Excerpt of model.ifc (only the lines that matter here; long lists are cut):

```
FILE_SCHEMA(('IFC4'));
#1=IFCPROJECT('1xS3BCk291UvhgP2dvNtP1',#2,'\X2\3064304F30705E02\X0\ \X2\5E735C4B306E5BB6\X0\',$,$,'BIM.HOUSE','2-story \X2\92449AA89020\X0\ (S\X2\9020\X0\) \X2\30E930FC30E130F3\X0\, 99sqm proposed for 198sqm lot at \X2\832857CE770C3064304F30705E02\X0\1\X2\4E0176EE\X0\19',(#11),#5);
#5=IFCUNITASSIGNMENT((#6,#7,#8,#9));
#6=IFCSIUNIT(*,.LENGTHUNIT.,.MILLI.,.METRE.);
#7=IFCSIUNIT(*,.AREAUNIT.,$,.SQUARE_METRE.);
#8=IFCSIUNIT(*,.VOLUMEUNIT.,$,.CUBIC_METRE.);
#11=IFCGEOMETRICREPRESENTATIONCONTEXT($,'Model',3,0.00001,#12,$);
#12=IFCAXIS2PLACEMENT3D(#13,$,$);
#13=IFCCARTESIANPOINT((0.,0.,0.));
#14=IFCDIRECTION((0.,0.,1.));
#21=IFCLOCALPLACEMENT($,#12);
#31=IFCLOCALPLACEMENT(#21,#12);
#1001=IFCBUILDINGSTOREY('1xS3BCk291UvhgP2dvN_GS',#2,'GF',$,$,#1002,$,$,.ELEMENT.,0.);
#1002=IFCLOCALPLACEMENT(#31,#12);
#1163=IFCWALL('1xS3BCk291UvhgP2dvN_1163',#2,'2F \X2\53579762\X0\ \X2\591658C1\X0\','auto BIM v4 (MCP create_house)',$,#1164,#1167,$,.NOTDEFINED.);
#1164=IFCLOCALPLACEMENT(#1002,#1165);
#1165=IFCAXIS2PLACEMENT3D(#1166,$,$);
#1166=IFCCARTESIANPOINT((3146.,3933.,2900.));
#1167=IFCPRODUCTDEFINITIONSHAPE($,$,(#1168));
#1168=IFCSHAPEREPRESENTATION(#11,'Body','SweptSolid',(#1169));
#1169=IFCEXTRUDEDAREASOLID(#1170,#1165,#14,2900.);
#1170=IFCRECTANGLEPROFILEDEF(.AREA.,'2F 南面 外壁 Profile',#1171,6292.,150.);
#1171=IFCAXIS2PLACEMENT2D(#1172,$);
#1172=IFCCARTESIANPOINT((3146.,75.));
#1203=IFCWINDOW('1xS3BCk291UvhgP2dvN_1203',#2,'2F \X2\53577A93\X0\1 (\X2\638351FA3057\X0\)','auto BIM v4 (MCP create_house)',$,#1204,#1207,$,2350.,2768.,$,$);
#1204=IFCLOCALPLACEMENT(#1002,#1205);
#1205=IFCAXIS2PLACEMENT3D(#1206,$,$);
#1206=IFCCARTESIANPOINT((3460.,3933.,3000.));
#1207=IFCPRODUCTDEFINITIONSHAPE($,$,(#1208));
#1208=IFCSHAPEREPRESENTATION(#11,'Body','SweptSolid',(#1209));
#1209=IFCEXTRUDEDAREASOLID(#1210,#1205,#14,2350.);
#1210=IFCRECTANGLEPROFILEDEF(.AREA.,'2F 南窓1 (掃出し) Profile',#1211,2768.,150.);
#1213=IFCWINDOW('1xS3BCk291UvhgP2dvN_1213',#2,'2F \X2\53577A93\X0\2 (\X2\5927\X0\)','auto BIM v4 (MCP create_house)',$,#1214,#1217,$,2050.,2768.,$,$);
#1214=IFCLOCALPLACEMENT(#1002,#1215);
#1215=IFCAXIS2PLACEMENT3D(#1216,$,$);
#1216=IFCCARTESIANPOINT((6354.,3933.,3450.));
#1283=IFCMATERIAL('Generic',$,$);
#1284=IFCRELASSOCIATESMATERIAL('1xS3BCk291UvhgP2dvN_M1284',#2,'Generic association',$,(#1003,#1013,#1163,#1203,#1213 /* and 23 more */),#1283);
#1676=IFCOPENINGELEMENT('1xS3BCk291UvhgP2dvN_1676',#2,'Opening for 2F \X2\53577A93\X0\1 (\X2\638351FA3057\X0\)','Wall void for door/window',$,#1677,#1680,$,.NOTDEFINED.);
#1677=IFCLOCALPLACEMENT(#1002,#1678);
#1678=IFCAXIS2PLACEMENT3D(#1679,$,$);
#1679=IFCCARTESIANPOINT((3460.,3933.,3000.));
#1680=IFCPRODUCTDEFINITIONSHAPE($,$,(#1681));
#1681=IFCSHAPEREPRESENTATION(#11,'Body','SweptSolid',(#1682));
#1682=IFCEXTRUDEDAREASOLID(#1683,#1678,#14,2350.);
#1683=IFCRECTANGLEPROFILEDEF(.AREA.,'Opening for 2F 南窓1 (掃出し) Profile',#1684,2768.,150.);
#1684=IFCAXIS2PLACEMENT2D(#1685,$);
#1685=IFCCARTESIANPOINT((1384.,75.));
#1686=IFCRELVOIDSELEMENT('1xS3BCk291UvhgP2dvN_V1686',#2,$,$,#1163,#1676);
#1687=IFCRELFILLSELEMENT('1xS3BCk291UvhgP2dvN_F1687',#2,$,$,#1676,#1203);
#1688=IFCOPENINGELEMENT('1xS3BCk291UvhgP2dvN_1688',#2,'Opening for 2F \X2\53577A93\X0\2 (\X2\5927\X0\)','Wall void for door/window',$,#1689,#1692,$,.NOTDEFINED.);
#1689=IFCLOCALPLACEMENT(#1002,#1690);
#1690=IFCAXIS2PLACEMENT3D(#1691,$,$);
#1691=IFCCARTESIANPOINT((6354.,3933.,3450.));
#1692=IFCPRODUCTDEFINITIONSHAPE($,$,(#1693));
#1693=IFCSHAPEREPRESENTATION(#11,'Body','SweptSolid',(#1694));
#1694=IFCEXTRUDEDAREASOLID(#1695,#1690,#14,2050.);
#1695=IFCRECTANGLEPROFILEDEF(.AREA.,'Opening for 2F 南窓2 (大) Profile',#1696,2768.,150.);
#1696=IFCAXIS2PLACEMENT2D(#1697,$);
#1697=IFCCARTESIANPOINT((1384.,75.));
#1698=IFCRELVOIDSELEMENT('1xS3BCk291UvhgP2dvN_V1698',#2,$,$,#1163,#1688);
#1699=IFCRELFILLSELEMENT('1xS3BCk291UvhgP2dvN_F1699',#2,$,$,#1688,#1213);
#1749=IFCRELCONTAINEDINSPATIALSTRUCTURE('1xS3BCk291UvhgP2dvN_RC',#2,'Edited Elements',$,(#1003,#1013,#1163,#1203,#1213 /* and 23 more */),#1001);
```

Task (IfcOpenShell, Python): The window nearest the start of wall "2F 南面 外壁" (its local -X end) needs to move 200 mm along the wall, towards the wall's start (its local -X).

```python
import ifcopenshell
import ifcopenshell.api.geometry
import ifcopenshell.util.placement
import ifcopenshell.util.unit

model = ifcopenshell.open("model.ifc")
unit_scale = ifcopenshell.util.unit.calculate_unit_scale(model)

window = model.by_guid("1xS3BCk291UvhgP2dvN_1203")
opening = window.FillsVoids[0].RelatingOpeningElement
wall = opening.VoidsElements[0].RelatingBuildingElement

wall_matrix = ifcopenshell.util.placement.get_local_placement(wall.ObjectPlacement)
shift = wall_matrix[:3, 0] * -0.2 / unit_scale
before = ifcopenshell.util.placement.get_local_placement(window.ObjectPlacement)[:3, 3].copy()

# The window is not placed relative to its opening, so move both.
for product in (opening, window):
    matrix = ifcopenshell.util.placement.get_local_placement(product.ObjectPlacement)
    matrix[:3, 3] += shift
    ifcopenshell.api.geometry.edit_object_placement(model, product=product, matrix=matrix, is_si=False)

after = ifcopenshell.util.placement.get_local_placement(window.ObjectPlacement)[:3, 3]
print("window moved by", (after - before).round(3) + 0.0)

model.write("model_rev.ifc")
```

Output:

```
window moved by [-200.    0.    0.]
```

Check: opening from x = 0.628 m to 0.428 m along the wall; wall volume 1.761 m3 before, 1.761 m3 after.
